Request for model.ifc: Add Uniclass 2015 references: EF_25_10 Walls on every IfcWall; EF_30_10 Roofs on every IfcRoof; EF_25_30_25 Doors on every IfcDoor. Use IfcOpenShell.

First a look at what the model holds.

```python
import ifcopenshell

model = ifcopenshell.open("model.ifc")
print(model.schema)
print("classifications:", [c.Name for c in model.by_type("IfcClassification")])
for ifc_class in ("IfcDoor", "IfcRoof", "IfcStair", "IfcWall", "IfcWindow"):
    print(ifc_class, len(model.by_type(ifc_class)))
```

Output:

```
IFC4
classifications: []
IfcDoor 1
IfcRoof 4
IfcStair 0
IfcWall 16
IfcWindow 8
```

```python
import ifcopenshell
import ifcopenshell.api.classification

model = ifcopenshell.open("model.ifc")

system = ifcopenshell.api.classification.add_classification(model, classification="Uniclass 2015")

codes = {
    "IfcWall": ("EF_25_10", "Walls"),
    "IfcRoof": ("EF_30_10", "Roofs"),
    "IfcDoor": ("EF_25_30_25", "Doors"),
}
for ifc_class, (code, name) in codes.items():
    products = model.by_type(ifc_class)
    ifcopenshell.api.classification.add_reference(
        model, products=products, classification=system, identification=code, name=name
    )
    print(code, len(products))

model.write("model_updated.ifc")
```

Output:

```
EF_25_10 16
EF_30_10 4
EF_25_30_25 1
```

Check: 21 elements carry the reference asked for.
